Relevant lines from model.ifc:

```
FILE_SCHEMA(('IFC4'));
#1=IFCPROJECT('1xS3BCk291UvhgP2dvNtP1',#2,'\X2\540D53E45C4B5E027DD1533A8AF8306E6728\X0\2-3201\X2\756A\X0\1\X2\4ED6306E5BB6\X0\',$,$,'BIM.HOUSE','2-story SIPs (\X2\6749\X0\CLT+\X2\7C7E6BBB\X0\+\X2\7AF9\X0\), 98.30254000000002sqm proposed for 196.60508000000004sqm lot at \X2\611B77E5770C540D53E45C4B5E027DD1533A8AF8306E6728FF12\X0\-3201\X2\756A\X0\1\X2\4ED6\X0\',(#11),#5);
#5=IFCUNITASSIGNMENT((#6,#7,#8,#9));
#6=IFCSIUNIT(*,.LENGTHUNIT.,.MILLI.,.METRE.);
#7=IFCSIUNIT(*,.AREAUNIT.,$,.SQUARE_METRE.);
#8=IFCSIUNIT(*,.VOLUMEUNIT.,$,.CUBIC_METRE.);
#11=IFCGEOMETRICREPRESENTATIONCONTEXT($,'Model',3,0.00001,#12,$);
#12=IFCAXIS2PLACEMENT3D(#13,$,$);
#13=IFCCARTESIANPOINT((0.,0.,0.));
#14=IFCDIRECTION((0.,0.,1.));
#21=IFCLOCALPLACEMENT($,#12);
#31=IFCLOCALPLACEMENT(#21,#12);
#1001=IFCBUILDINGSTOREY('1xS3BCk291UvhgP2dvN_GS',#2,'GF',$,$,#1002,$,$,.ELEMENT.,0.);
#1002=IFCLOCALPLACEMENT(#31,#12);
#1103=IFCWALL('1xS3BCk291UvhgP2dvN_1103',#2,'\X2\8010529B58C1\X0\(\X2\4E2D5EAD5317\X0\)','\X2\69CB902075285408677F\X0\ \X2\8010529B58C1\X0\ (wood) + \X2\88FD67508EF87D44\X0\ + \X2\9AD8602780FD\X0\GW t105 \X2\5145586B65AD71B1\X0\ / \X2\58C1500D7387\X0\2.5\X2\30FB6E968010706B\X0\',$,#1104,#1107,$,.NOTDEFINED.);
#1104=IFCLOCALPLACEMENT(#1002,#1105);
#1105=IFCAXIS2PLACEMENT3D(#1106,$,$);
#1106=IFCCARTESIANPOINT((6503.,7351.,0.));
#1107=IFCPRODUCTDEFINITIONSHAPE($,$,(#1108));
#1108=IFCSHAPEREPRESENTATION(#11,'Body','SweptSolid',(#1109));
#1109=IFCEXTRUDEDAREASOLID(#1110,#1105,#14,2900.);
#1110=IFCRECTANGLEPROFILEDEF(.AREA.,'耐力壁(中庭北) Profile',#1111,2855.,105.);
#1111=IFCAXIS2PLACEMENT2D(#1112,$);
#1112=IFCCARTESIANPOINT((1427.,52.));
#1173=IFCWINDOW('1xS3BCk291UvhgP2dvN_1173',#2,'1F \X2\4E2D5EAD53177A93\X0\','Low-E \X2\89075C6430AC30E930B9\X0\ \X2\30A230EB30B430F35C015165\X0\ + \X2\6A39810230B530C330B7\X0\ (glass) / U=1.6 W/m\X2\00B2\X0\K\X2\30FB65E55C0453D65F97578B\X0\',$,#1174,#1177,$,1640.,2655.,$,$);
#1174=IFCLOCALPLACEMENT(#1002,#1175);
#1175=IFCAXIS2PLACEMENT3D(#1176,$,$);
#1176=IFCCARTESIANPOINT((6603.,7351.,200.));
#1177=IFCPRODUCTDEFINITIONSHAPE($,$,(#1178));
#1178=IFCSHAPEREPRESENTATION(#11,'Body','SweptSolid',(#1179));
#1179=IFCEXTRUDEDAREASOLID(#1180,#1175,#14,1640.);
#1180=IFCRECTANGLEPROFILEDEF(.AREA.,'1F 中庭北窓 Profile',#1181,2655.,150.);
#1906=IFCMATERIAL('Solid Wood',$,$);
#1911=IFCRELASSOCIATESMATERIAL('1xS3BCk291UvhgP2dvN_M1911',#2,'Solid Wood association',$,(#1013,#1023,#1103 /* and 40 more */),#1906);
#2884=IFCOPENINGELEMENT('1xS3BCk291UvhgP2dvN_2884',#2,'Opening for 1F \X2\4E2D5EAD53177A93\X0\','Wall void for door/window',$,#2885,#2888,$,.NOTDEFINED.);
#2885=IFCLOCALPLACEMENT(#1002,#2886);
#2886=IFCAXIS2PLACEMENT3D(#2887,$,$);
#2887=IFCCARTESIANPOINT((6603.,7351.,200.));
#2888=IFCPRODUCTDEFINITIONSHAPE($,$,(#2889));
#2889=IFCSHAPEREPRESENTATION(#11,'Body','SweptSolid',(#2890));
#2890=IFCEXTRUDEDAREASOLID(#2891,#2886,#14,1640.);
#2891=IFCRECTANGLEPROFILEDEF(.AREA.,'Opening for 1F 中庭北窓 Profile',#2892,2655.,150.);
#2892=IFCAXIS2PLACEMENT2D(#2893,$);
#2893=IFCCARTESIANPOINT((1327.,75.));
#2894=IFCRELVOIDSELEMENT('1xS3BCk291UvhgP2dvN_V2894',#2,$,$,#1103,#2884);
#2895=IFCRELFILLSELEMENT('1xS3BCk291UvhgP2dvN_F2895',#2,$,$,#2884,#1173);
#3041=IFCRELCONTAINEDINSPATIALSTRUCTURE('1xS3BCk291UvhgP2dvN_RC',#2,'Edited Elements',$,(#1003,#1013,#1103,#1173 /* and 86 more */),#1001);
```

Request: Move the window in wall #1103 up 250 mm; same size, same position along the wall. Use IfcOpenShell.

```python
import numpy as np
import ifcopenshell
import ifcopenshell.api.geometry
import ifcopenshell.util.placement
import ifcopenshell.util.unit

model = ifcopenshell.open("model.ifc")
unit_scale = ifcopenshell.util.unit.calculate_unit_scale(model)

window = model.by_guid("1xS3BCk291UvhgP2dvN_1173")
opening = window.FillsVoids[0].RelatingOpeningElement
dz = 0.25 / unit_scale

shift = np.array([0.0, 0.0, dz])
# The window is not placed relative to its opening, so move both.
for product in (opening, window):
    matrix = ifcopenshell.util.placement.get_local_placement(product.ObjectPlacement)
    matrix[:3, 3] += shift
    ifcopenshell.api.geometry.edit_object_placement(model, product=product, matrix=matrix, is_si=False)

print(f"moved by {dz * unit_scale:+.3f} m")

model.write("model-out.ifc")
```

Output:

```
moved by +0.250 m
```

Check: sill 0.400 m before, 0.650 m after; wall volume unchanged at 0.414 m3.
